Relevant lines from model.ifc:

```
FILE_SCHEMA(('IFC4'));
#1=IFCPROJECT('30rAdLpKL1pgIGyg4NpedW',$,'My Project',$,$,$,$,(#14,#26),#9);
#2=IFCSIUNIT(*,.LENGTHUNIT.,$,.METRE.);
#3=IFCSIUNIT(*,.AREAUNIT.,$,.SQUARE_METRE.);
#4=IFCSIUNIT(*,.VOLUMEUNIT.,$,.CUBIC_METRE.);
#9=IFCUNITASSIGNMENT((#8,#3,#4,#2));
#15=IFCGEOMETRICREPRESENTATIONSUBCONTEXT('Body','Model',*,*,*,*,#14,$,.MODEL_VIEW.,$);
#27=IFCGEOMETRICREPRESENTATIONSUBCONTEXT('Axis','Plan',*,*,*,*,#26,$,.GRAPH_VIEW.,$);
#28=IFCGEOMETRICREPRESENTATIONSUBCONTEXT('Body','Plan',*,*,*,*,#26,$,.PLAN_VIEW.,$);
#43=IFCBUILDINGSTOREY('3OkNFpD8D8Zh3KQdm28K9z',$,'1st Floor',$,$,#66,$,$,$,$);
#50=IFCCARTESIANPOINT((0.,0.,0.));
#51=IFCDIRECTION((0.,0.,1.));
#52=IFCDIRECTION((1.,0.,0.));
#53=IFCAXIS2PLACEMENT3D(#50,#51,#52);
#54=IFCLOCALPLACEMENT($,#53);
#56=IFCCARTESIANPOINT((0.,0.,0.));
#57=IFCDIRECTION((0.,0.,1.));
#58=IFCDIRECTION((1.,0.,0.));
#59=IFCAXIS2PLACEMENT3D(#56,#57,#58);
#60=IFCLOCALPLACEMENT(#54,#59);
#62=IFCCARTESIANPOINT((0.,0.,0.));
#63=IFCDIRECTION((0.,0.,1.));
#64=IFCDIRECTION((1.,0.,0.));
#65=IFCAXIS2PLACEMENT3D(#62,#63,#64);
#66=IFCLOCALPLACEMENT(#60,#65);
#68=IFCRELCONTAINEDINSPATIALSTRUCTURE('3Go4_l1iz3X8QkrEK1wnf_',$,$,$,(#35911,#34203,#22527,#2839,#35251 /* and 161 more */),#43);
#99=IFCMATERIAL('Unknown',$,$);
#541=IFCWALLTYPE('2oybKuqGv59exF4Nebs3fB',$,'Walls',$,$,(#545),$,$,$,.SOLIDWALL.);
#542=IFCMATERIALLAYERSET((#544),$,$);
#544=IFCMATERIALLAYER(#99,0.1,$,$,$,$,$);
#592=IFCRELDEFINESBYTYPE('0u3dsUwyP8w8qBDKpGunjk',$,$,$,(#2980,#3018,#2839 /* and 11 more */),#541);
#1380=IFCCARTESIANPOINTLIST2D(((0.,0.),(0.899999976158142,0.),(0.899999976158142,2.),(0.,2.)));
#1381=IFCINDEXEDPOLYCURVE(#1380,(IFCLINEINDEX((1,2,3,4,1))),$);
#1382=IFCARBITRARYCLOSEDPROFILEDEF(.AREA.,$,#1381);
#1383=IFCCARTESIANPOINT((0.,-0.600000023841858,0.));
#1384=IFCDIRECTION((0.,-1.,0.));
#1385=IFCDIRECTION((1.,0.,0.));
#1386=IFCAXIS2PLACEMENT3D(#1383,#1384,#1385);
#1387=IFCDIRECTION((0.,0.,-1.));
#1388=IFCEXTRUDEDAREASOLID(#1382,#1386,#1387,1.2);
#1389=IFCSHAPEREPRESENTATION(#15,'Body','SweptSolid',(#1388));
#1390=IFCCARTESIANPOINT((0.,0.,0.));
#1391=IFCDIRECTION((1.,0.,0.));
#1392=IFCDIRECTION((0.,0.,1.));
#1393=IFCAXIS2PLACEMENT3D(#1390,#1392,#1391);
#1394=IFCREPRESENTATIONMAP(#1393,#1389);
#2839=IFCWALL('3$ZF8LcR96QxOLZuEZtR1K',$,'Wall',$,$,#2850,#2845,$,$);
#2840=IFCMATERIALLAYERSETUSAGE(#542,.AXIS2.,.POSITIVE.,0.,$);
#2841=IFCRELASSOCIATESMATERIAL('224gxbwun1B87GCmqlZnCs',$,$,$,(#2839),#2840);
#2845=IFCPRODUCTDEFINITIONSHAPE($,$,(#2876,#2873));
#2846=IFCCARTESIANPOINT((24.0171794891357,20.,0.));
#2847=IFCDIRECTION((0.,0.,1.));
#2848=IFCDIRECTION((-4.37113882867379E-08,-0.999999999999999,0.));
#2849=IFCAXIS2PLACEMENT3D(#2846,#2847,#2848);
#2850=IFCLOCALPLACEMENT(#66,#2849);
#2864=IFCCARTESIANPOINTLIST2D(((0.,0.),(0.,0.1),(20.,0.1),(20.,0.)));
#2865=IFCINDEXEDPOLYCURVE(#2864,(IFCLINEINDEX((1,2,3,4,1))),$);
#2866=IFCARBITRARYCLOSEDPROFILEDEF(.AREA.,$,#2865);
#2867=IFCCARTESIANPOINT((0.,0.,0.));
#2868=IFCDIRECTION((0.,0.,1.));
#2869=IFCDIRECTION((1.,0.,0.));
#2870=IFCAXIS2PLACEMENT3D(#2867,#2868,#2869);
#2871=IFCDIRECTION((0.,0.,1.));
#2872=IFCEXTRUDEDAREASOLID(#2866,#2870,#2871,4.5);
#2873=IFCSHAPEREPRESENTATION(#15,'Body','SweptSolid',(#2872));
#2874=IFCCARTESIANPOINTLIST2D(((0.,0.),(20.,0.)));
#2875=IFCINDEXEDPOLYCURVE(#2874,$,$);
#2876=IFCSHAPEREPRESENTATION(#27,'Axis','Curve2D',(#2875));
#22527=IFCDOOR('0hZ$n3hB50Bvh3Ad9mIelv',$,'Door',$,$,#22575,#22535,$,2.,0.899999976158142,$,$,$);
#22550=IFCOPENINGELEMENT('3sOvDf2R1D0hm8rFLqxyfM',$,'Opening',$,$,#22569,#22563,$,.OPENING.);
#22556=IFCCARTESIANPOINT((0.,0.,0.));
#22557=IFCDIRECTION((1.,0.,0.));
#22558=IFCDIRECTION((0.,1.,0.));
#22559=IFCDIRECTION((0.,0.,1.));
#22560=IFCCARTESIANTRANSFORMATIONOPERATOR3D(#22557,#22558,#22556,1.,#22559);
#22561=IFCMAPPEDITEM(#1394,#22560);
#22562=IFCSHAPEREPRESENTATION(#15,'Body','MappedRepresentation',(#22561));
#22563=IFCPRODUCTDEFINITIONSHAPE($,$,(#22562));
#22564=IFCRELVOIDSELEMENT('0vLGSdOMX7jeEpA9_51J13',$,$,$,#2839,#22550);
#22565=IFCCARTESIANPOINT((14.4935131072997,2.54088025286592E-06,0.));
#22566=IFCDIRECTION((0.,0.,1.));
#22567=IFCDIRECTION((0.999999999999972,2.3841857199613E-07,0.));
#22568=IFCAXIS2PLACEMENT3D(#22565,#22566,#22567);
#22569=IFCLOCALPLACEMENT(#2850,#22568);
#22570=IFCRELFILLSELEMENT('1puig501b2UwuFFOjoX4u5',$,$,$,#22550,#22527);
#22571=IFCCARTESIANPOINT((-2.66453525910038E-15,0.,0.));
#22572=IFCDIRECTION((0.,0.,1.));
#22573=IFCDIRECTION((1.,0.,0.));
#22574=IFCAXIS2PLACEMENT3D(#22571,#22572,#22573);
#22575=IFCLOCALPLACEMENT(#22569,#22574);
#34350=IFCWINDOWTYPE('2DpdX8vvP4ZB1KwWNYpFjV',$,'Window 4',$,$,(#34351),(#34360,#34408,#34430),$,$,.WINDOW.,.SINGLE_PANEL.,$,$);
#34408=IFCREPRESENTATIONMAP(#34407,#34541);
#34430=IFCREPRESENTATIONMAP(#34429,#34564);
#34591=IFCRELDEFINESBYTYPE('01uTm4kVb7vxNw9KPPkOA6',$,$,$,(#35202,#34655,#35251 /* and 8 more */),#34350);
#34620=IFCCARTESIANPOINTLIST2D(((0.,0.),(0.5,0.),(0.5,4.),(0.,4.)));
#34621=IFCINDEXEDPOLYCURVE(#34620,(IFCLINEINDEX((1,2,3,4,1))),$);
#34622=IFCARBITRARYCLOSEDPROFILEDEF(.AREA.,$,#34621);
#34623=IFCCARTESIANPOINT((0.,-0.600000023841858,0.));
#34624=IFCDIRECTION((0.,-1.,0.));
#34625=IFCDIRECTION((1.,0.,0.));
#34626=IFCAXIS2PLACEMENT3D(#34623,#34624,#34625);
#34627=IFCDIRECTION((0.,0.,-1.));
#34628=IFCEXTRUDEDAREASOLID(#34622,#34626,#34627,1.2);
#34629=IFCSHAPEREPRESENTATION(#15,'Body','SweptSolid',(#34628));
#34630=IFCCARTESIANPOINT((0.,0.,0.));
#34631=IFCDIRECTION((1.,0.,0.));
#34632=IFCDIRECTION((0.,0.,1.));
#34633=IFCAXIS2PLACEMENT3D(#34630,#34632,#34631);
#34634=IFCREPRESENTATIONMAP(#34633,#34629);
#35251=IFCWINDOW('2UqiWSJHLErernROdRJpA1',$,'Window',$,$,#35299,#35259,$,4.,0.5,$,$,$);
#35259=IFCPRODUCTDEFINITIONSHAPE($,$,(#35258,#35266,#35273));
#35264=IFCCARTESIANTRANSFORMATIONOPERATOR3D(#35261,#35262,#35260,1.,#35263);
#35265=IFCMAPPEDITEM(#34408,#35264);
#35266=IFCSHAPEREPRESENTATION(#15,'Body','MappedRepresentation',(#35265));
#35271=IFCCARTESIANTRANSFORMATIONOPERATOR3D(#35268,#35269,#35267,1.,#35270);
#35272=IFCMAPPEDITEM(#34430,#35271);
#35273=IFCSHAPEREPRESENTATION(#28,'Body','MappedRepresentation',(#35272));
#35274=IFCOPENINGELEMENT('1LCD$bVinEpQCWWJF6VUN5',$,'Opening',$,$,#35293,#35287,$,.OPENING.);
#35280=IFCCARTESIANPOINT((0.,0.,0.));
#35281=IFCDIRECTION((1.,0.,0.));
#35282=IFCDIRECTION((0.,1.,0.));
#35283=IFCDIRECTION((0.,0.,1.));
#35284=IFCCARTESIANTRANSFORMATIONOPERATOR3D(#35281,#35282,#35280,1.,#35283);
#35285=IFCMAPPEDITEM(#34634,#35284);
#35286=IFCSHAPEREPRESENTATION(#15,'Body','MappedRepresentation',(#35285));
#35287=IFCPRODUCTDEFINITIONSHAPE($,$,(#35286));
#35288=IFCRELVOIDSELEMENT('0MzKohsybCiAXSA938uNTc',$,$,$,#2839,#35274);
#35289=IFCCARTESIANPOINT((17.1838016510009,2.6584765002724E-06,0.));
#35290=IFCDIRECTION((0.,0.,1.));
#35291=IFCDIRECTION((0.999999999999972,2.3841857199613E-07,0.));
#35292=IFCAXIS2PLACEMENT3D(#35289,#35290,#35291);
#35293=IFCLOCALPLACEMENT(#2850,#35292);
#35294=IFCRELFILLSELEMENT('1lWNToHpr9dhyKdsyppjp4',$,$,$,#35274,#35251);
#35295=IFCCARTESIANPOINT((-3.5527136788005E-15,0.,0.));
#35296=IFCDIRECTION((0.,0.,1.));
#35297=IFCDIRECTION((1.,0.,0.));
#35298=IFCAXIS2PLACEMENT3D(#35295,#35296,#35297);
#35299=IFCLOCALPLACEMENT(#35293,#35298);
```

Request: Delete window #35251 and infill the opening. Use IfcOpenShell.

```python
import ifcopenshell
import ifcopenshell.api.feature
import ifcopenshell.api.root
import ifcopenshell.geom
import ifcopenshell.util.shape

model = ifcopenshell.open("model.ifc")
settings = ifcopenshell.geom.settings()


def volume(element):
    """Net volume in cubic metres, openings subtracted."""
    shape = ifcopenshell.geom.create_shape(settings, element)
    return ifcopenshell.util.shape.get_volume(shape.geometry)


window = model.by_guid("2UqiWSJHLErernROdRJpA1")
opening = window.FillsVoids[0].RelatingOpeningElement
wall = opening.VoidsElements[0].RelatingBuildingElement
before = volume(wall)

ifcopenshell.api.root.remove_product(model, product=window)
ifcopenshell.api.feature.remove_feature(model, feature=opening)

after = volume(wall)

print(f"wall volume {before:.3f} -> {after:.3f} m3")

model.write("model-out.ifc")
```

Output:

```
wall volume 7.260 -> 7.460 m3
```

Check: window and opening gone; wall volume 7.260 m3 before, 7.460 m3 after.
